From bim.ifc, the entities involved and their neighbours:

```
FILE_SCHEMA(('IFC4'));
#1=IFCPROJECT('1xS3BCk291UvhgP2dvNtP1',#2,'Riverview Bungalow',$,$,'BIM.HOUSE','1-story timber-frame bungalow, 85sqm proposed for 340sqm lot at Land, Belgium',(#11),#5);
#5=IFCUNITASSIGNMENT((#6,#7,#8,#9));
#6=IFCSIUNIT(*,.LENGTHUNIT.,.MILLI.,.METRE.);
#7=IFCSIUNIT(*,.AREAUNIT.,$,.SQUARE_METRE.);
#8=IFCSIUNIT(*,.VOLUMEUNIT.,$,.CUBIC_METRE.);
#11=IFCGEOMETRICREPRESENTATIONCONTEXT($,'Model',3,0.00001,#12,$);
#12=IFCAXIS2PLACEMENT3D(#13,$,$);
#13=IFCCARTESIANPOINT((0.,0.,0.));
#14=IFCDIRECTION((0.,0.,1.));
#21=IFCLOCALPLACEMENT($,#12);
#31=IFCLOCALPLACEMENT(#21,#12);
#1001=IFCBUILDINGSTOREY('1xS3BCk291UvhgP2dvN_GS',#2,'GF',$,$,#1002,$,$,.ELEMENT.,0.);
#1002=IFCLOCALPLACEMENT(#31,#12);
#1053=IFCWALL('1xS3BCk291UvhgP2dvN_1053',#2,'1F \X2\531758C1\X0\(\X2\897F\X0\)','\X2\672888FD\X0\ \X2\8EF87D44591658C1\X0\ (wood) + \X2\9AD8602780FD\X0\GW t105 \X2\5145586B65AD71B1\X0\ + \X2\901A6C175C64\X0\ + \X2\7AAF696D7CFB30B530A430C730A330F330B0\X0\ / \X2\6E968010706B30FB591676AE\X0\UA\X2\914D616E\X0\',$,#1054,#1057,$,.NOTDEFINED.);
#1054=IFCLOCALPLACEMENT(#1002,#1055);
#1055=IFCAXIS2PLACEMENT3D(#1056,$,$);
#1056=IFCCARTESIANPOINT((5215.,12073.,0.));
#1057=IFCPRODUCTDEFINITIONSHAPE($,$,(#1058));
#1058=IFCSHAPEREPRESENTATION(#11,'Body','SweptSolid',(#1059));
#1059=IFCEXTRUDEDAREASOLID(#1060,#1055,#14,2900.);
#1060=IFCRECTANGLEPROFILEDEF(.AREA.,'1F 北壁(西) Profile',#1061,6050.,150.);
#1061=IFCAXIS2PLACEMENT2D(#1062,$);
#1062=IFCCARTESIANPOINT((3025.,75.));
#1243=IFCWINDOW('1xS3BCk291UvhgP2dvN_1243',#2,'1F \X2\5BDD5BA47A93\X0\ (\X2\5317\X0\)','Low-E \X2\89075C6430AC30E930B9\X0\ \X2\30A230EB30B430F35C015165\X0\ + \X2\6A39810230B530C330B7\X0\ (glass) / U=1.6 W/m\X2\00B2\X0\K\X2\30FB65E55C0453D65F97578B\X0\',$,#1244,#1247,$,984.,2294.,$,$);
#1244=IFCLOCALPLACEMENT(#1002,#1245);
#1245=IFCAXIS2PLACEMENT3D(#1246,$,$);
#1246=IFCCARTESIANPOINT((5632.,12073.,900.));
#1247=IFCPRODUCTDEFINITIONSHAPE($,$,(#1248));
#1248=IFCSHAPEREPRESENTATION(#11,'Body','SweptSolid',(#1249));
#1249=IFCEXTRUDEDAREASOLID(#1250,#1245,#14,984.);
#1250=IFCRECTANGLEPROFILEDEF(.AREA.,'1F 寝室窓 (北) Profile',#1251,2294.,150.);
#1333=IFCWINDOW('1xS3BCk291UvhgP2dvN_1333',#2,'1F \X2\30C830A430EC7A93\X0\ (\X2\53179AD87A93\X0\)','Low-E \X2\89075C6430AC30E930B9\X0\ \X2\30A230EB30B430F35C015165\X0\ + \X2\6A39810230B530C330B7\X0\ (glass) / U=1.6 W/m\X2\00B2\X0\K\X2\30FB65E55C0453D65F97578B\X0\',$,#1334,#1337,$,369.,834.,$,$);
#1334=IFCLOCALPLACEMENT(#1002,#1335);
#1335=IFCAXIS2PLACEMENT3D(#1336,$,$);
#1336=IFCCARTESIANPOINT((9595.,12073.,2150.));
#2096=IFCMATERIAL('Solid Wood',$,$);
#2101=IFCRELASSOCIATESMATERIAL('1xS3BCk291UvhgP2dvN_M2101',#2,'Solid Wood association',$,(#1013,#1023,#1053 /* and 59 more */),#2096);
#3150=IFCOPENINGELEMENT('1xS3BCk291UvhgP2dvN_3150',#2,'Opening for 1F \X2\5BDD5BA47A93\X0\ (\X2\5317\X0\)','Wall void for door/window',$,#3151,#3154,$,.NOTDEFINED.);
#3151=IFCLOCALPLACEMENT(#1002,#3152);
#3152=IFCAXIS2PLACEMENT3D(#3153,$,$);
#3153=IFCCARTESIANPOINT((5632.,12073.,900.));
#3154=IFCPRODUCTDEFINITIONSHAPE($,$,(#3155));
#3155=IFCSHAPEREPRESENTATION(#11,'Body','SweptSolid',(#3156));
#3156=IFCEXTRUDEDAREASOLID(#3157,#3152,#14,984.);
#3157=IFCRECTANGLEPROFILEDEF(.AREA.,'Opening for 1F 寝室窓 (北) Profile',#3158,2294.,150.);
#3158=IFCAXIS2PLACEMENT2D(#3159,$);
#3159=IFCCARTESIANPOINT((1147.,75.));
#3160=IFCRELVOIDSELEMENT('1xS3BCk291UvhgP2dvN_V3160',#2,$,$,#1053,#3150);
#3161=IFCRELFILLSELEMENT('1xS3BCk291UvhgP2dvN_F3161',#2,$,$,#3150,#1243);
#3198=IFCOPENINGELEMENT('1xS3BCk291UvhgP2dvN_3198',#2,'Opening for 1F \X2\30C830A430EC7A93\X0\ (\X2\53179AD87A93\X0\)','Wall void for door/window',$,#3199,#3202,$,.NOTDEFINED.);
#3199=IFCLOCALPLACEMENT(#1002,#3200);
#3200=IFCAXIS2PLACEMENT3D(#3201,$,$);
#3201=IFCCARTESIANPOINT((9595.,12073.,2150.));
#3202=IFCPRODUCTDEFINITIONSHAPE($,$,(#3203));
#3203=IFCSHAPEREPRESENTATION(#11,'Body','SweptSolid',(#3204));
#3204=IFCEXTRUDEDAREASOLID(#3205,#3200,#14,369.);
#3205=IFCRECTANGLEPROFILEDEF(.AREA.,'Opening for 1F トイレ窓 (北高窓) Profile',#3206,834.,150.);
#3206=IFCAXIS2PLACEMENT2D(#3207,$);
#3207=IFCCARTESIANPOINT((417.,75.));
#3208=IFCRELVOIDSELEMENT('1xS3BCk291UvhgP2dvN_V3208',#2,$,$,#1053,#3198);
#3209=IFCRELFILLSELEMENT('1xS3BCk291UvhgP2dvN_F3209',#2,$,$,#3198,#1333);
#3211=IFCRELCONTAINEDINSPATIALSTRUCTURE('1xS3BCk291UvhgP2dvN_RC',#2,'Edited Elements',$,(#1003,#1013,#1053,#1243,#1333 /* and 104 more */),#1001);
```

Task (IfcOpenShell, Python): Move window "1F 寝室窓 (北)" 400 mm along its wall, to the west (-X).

```python
import ifcopenshell
import ifcopenshell.api.geometry
import ifcopenshell.util.placement
import ifcopenshell.util.unit

model = ifcopenshell.open("bim.ifc")
unit_scale = ifcopenshell.util.unit.calculate_unit_scale(model)

window = model.by_guid("1xS3BCk291UvhgP2dvN_1243")
opening = window.FillsVoids[0].RelatingOpeningElement
wall = opening.VoidsElements[0].RelatingBuildingElement

wall_matrix = ifcopenshell.util.placement.get_local_placement(wall.ObjectPlacement)
shift = wall_matrix[:3, 0] * -0.4 / unit_scale
before = ifcopenshell.util.placement.get_local_placement(window.ObjectPlacement)[:3, 3].copy()

# The window is not placed relative to its opening, so move both.
for product in (opening, window):
    matrix = ifcopenshell.util.placement.get_local_placement(product.ObjectPlacement)
    matrix[:3, 3] += shift
    ifcopenshell.api.geometry.edit_object_placement(model, product=product, matrix=matrix, is_si=False)

after = ifcopenshell.util.placement.get_local_placement(window.ObjectPlacement)[:3, 3]
print("window moved by", (after - before).round(3) + 0.0)

model.write("bim_edited.ifc")
```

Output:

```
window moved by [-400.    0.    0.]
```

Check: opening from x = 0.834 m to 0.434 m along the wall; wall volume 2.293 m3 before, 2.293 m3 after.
